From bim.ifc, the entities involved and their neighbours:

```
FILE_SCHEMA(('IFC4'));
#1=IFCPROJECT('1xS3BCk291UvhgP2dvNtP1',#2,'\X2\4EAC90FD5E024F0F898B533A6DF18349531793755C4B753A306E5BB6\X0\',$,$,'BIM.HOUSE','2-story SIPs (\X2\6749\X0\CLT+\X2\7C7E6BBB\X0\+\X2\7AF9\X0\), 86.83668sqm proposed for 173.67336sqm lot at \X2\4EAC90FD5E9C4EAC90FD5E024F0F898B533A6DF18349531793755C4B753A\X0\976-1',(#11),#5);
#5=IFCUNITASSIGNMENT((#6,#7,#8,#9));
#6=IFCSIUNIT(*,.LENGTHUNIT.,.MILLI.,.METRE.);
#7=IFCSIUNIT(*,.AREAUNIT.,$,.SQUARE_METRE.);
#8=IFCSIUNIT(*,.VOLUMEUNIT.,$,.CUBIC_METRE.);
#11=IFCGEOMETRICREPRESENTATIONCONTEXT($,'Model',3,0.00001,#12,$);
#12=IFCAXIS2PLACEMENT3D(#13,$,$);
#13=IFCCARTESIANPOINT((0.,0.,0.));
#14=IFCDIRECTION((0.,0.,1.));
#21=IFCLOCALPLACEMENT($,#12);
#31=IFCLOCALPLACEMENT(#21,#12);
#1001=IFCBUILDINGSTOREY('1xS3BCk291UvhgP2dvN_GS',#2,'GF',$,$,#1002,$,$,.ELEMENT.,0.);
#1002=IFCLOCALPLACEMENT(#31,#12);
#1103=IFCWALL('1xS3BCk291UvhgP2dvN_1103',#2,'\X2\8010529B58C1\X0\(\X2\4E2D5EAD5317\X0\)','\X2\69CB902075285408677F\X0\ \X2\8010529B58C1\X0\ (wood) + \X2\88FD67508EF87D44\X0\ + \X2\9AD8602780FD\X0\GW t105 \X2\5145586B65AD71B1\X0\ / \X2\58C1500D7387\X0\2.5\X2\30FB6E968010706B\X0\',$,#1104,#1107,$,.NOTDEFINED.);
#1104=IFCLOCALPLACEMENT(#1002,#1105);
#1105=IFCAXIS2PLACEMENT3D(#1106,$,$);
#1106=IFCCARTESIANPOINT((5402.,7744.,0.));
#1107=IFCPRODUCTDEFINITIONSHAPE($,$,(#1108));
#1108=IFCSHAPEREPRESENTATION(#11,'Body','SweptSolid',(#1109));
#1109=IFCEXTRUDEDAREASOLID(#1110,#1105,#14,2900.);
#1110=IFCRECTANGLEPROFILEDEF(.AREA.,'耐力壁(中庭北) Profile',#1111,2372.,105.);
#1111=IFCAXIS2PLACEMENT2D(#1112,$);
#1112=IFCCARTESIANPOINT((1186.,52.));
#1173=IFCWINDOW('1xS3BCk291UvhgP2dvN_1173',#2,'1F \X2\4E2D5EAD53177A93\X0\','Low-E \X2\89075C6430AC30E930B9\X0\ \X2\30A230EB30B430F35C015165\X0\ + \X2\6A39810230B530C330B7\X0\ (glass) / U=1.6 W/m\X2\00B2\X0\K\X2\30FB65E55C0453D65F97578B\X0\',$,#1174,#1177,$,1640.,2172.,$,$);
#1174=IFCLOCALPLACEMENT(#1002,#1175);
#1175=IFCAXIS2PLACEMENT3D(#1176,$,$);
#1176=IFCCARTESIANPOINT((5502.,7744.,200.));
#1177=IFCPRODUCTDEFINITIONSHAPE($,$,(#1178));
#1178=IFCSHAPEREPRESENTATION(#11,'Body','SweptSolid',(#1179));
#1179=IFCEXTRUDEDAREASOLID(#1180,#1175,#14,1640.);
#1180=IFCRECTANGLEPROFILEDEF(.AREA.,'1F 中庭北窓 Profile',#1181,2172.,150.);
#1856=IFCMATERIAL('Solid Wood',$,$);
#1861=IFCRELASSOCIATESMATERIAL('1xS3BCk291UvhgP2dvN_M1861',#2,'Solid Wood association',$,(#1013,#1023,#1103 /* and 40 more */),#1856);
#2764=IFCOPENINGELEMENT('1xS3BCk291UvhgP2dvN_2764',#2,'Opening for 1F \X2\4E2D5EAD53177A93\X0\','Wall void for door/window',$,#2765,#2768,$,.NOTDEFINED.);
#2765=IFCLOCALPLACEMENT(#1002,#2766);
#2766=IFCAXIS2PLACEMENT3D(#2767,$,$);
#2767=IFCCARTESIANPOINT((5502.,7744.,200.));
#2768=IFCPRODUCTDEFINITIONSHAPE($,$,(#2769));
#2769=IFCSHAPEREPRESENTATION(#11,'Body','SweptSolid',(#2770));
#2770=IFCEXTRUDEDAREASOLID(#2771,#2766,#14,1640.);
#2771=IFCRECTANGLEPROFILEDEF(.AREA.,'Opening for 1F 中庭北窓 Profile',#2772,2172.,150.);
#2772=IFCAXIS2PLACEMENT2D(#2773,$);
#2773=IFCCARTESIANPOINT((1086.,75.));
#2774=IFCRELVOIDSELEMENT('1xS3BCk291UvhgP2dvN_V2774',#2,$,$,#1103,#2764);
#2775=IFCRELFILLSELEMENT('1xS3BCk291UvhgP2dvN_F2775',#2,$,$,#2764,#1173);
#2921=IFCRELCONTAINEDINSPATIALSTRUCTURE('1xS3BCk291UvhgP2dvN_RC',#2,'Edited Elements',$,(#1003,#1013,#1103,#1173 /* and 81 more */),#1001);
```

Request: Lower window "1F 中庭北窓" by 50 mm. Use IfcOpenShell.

```python
import numpy as np
import ifcopenshell
import ifcopenshell.api.geometry
import ifcopenshell.util.placement
import ifcopenshell.util.unit

model = ifcopenshell.open("bim.ifc")
unit_scale = ifcopenshell.util.unit.calculate_unit_scale(model)

window = model.by_guid("1xS3BCk291UvhgP2dvN_1173")
opening = window.FillsVoids[0].RelatingOpeningElement
dz = -0.05 / unit_scale

shift = np.array([0.0, 0.0, dz])
# The window is not placed relative to its opening, so move both.
for product in (opening, window):
    matrix = ifcopenshell.util.placement.get_local_placement(product.ObjectPlacement)
    matrix[:3, 3] += shift
    ifcopenshell.api.geometry.edit_object_placement(model, product=product, matrix=matrix, is_si=False)

print(f"moved by {dz * unit_scale:+.3f} m")

model.write("bim-out.ifc")
```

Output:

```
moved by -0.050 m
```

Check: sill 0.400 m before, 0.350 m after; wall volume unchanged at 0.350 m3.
